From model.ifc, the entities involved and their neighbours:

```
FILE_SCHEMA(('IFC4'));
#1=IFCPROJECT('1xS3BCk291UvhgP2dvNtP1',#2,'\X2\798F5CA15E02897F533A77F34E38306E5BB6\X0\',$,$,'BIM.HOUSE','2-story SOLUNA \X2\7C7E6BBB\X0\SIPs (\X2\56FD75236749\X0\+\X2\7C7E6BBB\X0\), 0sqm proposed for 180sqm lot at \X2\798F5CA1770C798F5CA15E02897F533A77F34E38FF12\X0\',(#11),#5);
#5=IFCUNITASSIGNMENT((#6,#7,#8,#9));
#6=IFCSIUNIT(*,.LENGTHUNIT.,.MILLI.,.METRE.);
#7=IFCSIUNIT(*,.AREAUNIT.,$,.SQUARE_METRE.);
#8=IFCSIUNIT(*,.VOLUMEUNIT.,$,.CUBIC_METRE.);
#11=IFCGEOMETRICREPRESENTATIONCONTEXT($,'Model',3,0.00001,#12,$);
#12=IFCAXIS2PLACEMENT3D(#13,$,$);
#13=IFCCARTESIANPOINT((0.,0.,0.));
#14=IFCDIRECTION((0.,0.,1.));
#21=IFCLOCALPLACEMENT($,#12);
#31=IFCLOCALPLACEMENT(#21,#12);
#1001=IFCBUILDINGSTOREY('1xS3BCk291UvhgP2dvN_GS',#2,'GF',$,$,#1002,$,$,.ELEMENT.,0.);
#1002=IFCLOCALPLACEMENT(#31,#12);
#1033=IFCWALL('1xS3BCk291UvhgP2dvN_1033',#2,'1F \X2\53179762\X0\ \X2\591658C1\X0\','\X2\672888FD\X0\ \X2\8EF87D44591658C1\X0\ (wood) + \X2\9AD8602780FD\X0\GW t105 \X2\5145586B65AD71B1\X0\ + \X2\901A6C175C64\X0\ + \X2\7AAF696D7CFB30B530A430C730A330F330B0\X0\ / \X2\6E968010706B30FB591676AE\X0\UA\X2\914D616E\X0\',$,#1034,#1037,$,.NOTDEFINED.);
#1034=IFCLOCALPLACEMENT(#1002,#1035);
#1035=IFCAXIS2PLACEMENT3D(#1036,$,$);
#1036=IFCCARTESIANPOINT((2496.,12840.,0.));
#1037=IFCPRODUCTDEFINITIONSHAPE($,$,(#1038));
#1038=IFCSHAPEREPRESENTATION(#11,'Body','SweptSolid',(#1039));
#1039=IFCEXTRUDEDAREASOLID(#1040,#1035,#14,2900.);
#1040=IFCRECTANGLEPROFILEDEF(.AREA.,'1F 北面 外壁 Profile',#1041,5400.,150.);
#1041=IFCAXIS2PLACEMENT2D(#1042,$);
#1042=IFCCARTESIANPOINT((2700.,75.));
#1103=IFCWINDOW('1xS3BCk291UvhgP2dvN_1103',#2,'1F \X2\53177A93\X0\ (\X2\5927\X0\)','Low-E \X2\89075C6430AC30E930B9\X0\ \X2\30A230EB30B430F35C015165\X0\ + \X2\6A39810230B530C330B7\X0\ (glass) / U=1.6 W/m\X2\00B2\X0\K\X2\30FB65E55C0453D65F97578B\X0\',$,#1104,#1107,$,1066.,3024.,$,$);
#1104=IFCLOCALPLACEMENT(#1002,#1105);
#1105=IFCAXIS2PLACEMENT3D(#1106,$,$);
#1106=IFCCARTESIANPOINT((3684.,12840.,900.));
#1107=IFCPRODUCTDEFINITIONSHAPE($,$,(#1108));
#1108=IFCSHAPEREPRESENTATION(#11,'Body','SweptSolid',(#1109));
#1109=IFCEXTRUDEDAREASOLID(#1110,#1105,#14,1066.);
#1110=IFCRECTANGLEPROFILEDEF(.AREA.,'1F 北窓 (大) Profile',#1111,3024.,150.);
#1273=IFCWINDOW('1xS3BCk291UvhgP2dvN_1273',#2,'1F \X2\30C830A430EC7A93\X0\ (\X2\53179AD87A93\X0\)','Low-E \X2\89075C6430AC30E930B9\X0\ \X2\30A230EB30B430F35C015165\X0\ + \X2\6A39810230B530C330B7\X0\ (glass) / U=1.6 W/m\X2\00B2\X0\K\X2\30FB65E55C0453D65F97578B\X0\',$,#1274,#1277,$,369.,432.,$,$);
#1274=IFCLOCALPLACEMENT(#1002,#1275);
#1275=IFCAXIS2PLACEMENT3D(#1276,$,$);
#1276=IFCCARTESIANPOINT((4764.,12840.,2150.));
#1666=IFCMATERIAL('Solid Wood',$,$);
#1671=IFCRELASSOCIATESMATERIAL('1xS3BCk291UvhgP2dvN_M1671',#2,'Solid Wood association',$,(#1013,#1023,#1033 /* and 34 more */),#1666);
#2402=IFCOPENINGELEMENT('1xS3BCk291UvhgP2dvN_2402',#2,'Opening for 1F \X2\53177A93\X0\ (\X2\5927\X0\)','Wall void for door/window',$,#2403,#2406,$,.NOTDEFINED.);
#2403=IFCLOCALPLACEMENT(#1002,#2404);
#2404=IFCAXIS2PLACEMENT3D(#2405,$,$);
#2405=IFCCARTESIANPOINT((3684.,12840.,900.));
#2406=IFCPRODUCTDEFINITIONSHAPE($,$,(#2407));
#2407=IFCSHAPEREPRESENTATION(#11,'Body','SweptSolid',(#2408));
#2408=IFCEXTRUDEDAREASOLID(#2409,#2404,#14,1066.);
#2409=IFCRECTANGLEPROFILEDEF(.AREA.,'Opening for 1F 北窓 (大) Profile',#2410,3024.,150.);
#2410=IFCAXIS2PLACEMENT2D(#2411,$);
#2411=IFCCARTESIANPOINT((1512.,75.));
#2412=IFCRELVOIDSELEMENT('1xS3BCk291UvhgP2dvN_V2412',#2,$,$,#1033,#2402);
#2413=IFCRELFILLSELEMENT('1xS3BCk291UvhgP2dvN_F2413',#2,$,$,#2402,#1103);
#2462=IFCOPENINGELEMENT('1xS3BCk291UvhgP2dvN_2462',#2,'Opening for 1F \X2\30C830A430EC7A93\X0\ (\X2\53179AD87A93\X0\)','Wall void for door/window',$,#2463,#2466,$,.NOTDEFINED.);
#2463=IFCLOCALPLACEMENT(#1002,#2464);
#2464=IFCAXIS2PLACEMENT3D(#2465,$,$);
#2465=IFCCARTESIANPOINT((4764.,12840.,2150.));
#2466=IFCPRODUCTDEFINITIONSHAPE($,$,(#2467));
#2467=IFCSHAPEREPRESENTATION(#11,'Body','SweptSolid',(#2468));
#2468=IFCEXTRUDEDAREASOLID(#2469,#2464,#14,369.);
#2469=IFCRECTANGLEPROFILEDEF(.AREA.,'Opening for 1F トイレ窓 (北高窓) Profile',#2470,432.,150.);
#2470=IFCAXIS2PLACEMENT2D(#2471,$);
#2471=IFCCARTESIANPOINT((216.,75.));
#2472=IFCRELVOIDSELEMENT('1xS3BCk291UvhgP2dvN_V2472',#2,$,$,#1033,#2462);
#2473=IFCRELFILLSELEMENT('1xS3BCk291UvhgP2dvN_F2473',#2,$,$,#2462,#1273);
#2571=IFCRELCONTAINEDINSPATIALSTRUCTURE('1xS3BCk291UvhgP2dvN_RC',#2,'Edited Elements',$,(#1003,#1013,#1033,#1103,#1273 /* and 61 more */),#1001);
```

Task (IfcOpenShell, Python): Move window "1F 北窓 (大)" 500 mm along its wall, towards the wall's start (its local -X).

```python
import ifcopenshell
import ifcopenshell.api.geometry
import ifcopenshell.util.placement
import ifcopenshell.util.unit

model = ifcopenshell.open("model.ifc")
unit_scale = ifcopenshell.util.unit.calculate_unit_scale(model)

window = model.by_guid("1xS3BCk291UvhgP2dvN_1103")
opening = window.FillsVoids[0].RelatingOpeningElement
wall = opening.VoidsElements[0].RelatingBuildingElement

wall_matrix = ifcopenshell.util.placement.get_local_placement(wall.ObjectPlacement)
shift = wall_matrix[:3, 0] * -0.5 / unit_scale
before = ifcopenshell.util.placement.get_local_placement(window.ObjectPlacement)[:3, 3].copy()

# The window is not placed relative to its opening, so move both.
for product in (opening, window):
    matrix = ifcopenshell.util.placement.get_local_placement(product.ObjectPlacement)
    matrix[:3, 3] += shift
    ifcopenshell.api.geometry.edit_object_placement(model, product=product, matrix=matrix, is_si=False)

after = ifcopenshell.util.placement.get_local_placement(window.ObjectPlacement)[:3, 3]
print("window moved by", (after - before).round(3) + 0.0)

model.write("model_rev.ifc")
```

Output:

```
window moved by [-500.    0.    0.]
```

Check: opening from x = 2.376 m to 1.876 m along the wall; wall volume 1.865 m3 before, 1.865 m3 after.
